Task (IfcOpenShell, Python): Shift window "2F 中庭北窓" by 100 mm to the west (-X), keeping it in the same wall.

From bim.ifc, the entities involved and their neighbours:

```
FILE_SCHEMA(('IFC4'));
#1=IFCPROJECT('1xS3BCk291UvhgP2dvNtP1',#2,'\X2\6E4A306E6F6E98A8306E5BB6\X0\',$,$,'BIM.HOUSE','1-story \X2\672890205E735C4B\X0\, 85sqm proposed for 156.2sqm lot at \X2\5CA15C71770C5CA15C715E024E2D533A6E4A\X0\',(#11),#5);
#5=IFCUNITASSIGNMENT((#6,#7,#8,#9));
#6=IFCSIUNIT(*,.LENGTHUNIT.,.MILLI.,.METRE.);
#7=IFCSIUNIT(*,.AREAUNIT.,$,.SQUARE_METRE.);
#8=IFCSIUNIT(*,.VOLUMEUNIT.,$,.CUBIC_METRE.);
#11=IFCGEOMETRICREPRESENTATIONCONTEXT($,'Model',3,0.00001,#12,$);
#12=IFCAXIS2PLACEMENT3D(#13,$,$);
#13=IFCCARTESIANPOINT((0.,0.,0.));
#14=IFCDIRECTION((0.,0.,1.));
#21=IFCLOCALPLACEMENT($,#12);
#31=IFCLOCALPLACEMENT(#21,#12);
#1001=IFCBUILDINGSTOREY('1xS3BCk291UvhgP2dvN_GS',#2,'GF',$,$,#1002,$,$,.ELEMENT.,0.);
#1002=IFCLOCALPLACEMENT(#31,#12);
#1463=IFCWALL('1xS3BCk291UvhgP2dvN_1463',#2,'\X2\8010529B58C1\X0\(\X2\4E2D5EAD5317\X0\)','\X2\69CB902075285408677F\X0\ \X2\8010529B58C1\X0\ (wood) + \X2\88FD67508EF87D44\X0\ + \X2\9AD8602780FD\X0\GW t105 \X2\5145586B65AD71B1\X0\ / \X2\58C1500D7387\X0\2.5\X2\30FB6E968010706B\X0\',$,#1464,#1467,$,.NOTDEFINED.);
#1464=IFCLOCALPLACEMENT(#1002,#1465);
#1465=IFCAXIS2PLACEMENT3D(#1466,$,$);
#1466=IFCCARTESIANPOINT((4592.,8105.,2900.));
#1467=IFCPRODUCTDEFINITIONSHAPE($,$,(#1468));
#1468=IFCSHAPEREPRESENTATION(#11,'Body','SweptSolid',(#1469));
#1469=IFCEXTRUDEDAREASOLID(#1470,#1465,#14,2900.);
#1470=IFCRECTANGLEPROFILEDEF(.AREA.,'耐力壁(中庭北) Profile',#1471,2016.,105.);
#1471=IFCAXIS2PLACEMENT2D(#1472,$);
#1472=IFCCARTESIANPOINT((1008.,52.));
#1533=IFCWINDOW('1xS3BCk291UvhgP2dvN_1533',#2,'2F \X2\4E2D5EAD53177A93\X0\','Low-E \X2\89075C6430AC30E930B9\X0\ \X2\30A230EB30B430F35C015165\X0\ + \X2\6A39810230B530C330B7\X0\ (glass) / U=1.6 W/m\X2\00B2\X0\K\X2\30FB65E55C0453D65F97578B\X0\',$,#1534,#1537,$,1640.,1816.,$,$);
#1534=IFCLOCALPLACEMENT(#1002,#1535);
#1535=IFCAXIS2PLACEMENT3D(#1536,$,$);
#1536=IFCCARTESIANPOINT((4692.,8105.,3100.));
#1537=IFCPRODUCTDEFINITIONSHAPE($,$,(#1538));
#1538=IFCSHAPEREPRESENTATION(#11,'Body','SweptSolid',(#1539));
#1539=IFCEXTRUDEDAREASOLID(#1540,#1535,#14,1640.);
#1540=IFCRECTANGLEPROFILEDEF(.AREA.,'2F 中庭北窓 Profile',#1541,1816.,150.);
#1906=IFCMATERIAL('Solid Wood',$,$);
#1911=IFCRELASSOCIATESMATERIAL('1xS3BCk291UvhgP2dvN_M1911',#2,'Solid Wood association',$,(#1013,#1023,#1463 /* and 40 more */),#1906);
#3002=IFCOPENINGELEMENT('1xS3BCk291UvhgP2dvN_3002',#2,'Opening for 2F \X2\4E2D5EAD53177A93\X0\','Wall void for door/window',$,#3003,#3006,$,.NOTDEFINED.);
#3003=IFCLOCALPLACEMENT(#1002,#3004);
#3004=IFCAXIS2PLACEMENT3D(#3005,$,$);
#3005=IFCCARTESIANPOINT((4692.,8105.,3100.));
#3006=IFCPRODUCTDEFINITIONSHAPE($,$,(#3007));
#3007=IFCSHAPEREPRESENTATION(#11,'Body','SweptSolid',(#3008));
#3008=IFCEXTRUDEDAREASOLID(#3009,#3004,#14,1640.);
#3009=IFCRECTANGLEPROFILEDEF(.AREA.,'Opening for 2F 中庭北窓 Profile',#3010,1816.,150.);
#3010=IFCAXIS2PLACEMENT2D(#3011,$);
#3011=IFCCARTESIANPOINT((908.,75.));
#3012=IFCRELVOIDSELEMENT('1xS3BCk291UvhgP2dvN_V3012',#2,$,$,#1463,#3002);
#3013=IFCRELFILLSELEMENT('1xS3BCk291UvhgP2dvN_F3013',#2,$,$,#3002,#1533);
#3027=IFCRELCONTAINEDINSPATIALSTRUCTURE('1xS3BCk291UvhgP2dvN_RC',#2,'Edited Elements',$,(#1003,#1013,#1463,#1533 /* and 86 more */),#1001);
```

```python
import ifcopenshell
import ifcopenshell.api.geometry
import ifcopenshell.util.placement

model = ifcopenshell.open("bim.ifc")

window = model.by_guid("1xS3BCk291UvhgP2dvN_1533")
opening = window.FillsVoids[0].RelatingOpeningElement
wall = opening.VoidsElements[0].RelatingBuildingElement

wall_matrix = ifcopenshell.util.placement.get_local_placement(wall.ObjectPlacement)
shift = wall_matrix[:3, 0] * -100.0
before = ifcopenshell.util.placement.get_local_placement(window.ObjectPlacement)[:3, 3].copy()

# The window is not placed relative to its opening, so move both.
for product in (opening, window):
    matrix = ifcopenshell.util.placement.get_local_placement(product.ObjectPlacement)
    matrix[:3, 3] += shift
    ifcopenshell.api.geometry.edit_object_placement(model, product=product, matrix=matrix, is_si=False)

after = ifcopenshell.util.placement.get_local_placement(window.ObjectPlacement)[:3, 3]
print("window moved by", (after - before).round(3) + 0.0)

model.write("bim_v2.ifc")
```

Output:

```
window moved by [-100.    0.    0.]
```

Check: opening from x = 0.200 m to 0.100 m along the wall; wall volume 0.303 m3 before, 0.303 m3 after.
